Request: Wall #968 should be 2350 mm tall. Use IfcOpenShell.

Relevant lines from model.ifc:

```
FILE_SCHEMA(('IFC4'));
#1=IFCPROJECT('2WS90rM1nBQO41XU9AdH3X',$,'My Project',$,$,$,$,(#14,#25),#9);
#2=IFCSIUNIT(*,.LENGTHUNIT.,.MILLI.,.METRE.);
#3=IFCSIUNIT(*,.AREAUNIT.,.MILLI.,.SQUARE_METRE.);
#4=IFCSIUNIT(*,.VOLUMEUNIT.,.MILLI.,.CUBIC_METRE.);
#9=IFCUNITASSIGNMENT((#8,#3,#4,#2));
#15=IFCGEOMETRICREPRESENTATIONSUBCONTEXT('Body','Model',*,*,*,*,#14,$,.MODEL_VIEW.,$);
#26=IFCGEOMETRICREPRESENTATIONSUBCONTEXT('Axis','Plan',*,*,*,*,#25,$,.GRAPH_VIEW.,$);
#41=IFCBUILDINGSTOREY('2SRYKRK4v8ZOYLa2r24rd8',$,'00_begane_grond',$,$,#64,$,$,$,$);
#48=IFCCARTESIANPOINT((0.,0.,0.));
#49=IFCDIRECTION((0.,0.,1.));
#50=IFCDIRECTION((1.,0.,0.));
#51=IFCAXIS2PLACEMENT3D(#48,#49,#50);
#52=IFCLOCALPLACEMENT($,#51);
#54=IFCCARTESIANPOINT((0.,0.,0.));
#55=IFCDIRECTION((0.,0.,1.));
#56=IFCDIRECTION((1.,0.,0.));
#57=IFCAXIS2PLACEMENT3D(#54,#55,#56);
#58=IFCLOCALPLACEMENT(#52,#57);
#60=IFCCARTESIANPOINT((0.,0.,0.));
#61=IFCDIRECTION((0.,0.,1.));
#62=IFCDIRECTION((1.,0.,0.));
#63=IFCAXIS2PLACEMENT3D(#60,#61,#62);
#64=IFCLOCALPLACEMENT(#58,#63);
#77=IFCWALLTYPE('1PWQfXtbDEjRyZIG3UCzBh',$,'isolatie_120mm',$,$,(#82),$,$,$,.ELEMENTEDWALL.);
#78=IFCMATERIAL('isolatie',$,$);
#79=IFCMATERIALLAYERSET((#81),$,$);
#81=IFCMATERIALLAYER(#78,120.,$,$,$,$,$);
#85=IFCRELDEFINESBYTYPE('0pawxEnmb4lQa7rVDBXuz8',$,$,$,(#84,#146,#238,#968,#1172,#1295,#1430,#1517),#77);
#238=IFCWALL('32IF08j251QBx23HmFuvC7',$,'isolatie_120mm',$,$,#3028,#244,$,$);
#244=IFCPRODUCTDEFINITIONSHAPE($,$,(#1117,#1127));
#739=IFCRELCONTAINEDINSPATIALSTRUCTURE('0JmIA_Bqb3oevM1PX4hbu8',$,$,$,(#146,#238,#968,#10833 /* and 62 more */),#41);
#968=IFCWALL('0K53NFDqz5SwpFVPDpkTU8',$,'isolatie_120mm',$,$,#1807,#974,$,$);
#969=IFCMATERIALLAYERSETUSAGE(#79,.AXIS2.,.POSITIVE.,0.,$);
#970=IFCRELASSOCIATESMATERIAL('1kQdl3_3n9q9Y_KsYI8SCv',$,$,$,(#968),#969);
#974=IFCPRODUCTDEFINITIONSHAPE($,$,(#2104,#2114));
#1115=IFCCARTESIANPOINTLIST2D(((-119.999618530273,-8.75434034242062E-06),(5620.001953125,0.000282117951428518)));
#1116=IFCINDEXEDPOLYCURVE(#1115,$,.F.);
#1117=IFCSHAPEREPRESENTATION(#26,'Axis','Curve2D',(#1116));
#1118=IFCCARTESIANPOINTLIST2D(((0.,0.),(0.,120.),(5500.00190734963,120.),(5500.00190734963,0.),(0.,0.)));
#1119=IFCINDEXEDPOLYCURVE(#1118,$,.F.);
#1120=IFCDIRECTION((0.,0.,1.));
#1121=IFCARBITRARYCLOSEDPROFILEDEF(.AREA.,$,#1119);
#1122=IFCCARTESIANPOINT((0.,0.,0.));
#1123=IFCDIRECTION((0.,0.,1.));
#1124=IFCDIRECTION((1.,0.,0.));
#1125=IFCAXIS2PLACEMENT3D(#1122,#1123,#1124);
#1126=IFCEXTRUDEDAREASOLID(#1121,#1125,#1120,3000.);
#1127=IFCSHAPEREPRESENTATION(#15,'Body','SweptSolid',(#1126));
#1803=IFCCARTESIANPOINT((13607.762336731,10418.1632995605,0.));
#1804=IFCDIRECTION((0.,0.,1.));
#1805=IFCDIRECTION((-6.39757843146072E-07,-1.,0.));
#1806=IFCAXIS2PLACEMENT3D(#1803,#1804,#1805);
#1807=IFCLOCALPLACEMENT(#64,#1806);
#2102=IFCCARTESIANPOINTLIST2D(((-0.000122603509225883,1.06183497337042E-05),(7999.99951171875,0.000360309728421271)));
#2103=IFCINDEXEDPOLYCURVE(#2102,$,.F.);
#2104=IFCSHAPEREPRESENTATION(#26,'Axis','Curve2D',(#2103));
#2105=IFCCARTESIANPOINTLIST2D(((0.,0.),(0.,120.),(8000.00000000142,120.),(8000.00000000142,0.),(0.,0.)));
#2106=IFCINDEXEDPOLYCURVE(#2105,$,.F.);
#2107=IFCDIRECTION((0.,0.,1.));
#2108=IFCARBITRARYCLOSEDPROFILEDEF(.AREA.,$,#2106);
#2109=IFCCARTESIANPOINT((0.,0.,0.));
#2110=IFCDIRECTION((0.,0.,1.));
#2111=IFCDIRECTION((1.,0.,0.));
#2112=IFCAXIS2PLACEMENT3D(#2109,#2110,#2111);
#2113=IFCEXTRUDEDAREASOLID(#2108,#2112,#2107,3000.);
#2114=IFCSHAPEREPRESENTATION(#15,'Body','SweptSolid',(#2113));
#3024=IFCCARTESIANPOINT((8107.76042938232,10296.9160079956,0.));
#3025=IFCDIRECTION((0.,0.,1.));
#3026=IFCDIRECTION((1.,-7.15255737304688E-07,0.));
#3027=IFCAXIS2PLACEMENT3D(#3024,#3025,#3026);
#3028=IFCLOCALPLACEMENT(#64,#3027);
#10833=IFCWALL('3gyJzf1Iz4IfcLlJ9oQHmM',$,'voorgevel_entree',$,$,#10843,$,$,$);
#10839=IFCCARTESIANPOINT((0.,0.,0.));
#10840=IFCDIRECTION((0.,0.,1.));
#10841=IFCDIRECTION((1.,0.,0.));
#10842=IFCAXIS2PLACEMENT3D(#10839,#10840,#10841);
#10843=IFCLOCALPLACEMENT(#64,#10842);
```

```python
import ifcopenshell
import ifcopenshell.geom
import ifcopenshell.util.representation
import ifcopenshell.util.shape

model = ifcopenshell.open("model.ifc")
settings = ifcopenshell.geom.settings()


def volume(element):
    """Net volume in cubic metres, openings subtracted."""
    shape = ifcopenshell.geom.create_shape(settings, element)
    return ifcopenshell.util.shape.get_volume(shape.geometry)


wall = model.by_guid("0K53NFDqz5SwpFVPDpkTU8")
before = volume(wall)

body = ifcopenshell.util.representation.get_representation(wall, "Model", "Body")
solid = body.Items[0]
old_height = solid.Depth
solid.Depth = 2350.0
after = volume(wall)

print(f"height {old_height:g} -> {solid.Depth:g}, volume {before:.3f} -> {after:.3f} m3")

model.write("model_updated.ifc")
```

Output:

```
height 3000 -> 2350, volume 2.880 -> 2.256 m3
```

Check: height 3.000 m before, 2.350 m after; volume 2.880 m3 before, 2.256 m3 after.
